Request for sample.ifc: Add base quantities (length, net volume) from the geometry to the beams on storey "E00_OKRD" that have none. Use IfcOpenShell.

First a look at what the model holds.

```python
import ifcopenshell
import ifcopenshell.util.element
import ifcopenshell.util.unit

model = ifcopenshell.open("sample.ifc")
print(model.schema)
for unit_type in ("LENGTHUNIT", "AREAUNIT", "VOLUMEUNIT"):
    print(unit_type, ifcopenshell.util.unit.calculate_unit_scale(model, unit_type))
storey = next(s for s in model.by_type("IfcBuildingStorey") if s.Name == "E00_OKRD")
beams = [e for e in ifcopenshell.util.element.get_decomposition(storey) if e.is_a("IfcBeam")]
for e in sorted(beams, key=lambda e: e.id()):
    print(e.id(), e.is_a(), e.Name, list(ifcopenshell.util.element.get_psets(e, qtos_only=True)), sep=" | ")
```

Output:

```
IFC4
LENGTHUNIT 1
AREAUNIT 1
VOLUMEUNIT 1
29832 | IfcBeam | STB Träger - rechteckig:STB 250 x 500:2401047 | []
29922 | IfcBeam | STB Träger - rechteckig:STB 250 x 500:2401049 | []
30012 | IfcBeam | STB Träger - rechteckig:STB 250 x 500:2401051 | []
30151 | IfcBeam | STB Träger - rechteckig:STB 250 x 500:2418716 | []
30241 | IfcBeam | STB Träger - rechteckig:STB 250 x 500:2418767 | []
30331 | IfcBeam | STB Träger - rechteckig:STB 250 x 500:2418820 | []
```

```python
import ifcopenshell
import ifcopenshell.api.pset
import ifcopenshell.geom
import ifcopenshell.util.element
import ifcopenshell.util.shape
import ifcopenshell.util.unit

model = ifcopenshell.open("sample.ifc")
unit_scale = ifcopenshell.util.unit.calculate_unit_scale(model)
volume_scale = ifcopenshell.util.unit.calculate_unit_scale(model, "VOLUMEUNIT")
settings = ifcopenshell.geom.settings()

storey = next(s for s in model.by_type("IfcBuildingStorey") if s.Name == "E00_OKRD")
beams = [e for e in ifcopenshell.util.element.get_decomposition(storey) if e.is_a("IfcBeam")]

for e in sorted(beams, key=lambda e: e.id()):
    if ifcopenshell.util.element.get_psets(e, qtos_only=True, should_inherit=False):
        continue
    # Geometry comes back in metres, in the element's own axes.
    shape = ifcopenshell.geom.create_shape(settings, e)
    values = {
        "Length": ifcopenshell.util.shape.get_max_xyz(shape.geometry) / unit_scale,
        "NetVolume": ifcopenshell.util.shape.get_volume(shape.geometry) / volume_scale,
    }
    qto = ifcopenshell.api.pset.add_qto(model, product=e, name="Qto_BeamBaseQuantities")
    ifcopenshell.api.pset.edit_qto(model, qto=qto, properties=values)
    print(e.id(), {k: round(v, 3) for k, v in values.items()})

model.write("sample_rev.ifc")
```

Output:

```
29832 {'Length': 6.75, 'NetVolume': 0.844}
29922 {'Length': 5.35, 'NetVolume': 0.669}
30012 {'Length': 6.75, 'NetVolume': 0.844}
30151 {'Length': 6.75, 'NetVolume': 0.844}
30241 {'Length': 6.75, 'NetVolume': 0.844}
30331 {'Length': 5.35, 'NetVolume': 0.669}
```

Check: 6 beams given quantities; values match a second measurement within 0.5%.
